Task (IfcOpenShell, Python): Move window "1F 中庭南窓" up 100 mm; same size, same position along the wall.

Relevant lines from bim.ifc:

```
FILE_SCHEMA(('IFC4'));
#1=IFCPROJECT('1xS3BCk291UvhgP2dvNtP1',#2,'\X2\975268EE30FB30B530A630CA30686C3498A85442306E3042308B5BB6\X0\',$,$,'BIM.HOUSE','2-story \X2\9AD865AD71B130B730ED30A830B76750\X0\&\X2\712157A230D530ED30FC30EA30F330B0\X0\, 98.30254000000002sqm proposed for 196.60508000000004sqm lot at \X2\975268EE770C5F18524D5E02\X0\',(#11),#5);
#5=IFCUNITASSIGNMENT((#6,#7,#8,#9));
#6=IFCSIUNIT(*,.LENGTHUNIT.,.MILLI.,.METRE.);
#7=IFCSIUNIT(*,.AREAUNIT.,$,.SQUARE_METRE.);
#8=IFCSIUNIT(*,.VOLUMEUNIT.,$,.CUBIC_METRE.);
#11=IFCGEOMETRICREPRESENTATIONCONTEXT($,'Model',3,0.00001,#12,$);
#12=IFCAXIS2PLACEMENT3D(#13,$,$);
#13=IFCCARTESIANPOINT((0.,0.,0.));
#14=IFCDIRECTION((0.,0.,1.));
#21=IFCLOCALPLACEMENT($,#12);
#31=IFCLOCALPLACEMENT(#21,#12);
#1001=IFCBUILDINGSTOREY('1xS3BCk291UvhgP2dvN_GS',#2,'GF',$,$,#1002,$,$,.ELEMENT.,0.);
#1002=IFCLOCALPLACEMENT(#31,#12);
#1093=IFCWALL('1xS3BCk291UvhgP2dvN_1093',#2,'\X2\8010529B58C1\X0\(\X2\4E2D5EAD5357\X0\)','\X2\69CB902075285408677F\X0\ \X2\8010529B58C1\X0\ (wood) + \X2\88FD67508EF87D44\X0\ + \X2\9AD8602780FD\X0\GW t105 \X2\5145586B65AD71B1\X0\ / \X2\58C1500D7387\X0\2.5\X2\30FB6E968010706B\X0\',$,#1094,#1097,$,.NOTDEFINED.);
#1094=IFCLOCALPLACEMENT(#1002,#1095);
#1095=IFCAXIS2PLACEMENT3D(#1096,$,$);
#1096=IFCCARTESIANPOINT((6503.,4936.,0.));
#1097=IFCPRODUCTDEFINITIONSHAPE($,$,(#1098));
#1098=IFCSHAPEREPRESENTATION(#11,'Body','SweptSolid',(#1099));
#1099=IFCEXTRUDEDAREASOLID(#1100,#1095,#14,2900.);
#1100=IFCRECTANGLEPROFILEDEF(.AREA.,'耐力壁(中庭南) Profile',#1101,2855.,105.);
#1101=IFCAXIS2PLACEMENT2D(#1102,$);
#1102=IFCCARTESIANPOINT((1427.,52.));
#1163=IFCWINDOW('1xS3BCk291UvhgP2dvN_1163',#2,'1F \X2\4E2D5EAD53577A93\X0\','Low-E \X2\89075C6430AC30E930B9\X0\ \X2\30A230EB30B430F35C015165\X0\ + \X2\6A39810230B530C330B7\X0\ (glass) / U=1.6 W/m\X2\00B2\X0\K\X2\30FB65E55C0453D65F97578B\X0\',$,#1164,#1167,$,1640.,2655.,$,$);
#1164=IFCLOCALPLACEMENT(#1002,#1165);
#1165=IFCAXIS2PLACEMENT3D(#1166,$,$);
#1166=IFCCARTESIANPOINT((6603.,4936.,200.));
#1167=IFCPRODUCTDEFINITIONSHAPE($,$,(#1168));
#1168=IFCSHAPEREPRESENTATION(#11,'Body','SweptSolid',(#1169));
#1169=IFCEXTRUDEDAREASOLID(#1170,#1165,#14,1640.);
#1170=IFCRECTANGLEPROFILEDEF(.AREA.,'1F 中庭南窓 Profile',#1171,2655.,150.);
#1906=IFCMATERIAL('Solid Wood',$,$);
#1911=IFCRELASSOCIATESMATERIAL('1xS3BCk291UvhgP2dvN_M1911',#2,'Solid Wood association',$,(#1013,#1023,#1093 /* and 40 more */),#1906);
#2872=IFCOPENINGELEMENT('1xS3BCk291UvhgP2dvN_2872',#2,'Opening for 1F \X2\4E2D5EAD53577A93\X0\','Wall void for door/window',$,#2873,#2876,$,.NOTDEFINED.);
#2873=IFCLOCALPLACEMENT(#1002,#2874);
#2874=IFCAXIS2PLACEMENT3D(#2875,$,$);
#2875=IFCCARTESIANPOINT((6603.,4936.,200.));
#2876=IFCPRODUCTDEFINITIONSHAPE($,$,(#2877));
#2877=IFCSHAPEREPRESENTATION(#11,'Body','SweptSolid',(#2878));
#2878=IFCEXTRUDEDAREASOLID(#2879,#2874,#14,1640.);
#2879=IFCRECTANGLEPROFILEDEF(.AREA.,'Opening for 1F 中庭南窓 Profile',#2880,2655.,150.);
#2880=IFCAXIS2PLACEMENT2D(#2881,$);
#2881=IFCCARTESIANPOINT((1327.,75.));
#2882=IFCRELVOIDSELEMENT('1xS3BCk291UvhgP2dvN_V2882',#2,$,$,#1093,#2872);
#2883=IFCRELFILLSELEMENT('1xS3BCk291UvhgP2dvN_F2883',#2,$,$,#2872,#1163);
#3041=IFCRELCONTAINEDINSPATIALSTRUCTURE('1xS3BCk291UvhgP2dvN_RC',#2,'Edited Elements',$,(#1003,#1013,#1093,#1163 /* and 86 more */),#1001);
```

```python
import numpy as np
import ifcopenshell
import ifcopenshell.api.geometry
import ifcopenshell.util.placement
import ifcopenshell.util.unit

model = ifcopenshell.open("bim.ifc")
unit_scale = ifcopenshell.util.unit.calculate_unit_scale(model)

window = model.by_guid("1xS3BCk291UvhgP2dvN_1163")
opening = window.FillsVoids[0].RelatingOpeningElement
dz = 0.1 / unit_scale

shift = np.array([0.0, 0.0, dz])
# The window is not placed relative to its opening, so move both.
for product in (opening, window):
    matrix = ifcopenshell.util.placement.get_local_placement(product.ObjectPlacement)
    matrix[:3, 3] += shift
    ifcopenshell.api.geometry.edit_object_placement(model, product=product, matrix=matrix, is_si=False)

print(f"moved by {dz * unit_scale:+.3f} m")

model.write("bim_edited.ifc")
```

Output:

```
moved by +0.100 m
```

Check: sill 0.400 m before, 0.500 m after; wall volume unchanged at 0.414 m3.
